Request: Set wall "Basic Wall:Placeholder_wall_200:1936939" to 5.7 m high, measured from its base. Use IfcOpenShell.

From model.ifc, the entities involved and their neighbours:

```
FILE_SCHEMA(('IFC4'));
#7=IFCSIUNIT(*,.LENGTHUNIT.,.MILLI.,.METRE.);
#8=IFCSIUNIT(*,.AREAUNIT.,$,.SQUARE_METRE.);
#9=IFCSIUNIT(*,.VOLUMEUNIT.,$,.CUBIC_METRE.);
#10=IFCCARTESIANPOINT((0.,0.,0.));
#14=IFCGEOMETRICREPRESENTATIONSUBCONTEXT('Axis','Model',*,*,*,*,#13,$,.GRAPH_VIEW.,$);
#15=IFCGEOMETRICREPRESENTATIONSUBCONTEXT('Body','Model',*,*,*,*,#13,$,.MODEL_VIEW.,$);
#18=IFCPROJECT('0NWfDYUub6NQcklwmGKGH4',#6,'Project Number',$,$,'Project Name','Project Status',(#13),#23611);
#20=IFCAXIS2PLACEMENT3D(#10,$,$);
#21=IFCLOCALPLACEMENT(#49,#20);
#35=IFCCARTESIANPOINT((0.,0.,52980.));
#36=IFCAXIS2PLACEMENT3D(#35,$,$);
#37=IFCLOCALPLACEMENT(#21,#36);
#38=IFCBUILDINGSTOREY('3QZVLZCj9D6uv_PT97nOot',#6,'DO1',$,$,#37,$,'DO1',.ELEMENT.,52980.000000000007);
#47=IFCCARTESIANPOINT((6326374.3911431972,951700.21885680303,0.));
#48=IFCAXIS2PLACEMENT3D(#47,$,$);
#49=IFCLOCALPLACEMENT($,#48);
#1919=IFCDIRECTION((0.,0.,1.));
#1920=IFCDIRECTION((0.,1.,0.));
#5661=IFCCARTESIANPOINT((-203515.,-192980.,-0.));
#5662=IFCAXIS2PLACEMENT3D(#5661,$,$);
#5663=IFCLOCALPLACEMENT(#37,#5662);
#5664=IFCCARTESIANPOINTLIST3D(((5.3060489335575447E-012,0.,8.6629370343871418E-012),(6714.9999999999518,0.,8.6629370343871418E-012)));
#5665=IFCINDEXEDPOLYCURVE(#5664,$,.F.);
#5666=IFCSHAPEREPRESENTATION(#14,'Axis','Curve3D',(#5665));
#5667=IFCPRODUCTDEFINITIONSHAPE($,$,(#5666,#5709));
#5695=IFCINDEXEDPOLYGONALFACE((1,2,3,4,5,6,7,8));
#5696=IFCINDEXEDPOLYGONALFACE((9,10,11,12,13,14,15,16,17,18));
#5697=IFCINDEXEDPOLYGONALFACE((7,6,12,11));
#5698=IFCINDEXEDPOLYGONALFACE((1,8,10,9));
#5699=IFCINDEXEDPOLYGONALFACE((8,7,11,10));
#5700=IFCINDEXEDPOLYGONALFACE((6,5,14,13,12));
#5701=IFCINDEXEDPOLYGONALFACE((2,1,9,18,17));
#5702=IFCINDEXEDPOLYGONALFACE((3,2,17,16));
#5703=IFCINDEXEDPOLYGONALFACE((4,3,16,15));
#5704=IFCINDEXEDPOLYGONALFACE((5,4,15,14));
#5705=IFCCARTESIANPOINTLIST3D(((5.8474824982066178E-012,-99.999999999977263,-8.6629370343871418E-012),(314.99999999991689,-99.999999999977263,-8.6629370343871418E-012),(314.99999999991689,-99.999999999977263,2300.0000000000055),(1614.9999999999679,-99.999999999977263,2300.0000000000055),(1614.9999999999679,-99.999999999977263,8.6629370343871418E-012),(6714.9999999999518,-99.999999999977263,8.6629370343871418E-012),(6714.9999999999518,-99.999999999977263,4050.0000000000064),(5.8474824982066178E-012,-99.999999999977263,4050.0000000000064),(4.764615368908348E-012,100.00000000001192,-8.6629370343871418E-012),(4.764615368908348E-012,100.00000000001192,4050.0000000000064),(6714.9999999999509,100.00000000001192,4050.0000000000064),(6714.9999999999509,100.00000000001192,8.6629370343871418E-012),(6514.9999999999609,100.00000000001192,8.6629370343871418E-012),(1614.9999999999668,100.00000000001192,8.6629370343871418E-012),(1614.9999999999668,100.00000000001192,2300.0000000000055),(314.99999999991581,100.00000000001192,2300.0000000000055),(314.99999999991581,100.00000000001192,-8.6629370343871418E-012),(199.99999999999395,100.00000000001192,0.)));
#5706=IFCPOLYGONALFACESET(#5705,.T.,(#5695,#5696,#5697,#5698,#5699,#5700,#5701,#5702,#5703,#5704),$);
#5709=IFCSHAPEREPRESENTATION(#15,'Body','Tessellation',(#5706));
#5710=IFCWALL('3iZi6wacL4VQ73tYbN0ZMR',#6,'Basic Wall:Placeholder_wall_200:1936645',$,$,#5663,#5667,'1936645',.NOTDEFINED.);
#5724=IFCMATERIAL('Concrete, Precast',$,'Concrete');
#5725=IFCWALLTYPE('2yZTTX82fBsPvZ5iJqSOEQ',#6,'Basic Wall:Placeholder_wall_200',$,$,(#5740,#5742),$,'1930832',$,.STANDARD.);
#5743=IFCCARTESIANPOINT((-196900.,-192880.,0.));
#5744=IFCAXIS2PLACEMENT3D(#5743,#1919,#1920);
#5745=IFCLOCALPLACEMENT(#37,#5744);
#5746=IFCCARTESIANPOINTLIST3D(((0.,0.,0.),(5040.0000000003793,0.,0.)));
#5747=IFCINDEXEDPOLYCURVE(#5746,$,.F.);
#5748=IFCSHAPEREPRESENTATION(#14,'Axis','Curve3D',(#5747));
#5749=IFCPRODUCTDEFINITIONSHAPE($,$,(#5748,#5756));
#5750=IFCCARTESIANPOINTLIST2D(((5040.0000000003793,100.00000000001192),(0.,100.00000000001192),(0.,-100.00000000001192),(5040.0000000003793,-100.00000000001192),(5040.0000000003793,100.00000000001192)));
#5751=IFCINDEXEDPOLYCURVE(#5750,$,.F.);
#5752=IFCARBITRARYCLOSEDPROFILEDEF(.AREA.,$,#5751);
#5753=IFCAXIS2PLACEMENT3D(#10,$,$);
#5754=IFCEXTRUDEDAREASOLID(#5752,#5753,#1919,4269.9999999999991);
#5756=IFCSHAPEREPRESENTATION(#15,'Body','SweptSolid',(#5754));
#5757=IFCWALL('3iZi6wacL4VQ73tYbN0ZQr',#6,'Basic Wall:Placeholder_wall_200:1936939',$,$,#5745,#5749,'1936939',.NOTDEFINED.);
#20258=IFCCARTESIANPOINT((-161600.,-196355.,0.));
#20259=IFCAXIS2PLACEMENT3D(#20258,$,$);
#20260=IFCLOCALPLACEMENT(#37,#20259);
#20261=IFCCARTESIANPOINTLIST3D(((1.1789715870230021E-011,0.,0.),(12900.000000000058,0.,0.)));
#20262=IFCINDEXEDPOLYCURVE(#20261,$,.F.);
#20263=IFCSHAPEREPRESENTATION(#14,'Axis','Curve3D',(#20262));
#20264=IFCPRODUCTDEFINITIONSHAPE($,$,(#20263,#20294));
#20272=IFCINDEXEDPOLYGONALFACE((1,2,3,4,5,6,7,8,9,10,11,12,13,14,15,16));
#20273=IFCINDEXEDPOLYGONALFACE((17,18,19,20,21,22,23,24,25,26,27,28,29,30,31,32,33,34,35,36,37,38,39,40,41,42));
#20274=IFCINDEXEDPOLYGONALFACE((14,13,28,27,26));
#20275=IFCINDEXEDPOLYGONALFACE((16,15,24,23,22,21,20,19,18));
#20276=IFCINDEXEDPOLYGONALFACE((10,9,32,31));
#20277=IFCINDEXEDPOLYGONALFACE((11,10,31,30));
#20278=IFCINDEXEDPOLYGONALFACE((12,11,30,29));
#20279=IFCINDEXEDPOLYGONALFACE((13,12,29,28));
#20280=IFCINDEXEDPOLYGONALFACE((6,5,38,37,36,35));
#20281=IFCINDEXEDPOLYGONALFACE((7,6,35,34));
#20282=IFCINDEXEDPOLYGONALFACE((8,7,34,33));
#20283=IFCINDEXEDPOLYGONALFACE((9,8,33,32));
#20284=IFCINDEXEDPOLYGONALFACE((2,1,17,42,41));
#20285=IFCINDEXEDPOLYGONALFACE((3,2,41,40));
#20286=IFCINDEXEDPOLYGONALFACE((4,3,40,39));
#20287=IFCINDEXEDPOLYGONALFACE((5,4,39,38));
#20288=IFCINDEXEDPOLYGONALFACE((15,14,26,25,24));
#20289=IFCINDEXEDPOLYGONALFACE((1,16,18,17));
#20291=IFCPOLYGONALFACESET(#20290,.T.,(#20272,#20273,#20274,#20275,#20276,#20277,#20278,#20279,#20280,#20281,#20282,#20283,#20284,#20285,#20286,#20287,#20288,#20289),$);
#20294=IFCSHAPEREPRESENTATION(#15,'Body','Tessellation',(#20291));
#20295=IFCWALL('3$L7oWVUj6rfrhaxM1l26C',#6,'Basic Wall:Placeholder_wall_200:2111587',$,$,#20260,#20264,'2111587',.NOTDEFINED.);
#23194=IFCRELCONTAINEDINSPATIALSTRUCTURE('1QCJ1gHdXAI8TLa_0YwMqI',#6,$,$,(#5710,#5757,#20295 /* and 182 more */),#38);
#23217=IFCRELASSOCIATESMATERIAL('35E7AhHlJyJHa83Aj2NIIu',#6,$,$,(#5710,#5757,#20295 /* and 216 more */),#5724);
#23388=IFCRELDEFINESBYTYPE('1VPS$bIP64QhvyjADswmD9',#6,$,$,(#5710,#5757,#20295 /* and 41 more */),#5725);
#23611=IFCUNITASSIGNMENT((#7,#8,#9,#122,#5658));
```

```python
import ifcopenshell
import ifcopenshell.geom
import ifcopenshell.util.representation
import ifcopenshell.util.shape
import ifcopenshell.util.unit

model = ifcopenshell.open("model.ifc")
unit_scale = ifcopenshell.util.unit.calculate_unit_scale(model)
settings = ifcopenshell.geom.settings()


def volume(element):
    """Net volume in cubic metres, openings subtracted."""
    shape = ifcopenshell.geom.create_shape(settings, element)
    return ifcopenshell.util.shape.get_volume(shape.geometry)


wall = model.by_guid("3iZi6wacL4VQ73tYbN0ZQr")
before = volume(wall)

body = ifcopenshell.util.representation.get_representation(wall, "Model", "Body")
solid = body.Items[0]
old_height = solid.Depth
solid.Depth = 5.7 / unit_scale
after = volume(wall)

print(f"height {old_height:g} -> {solid.Depth:g}, volume {before:.3f} -> {after:.3f} m3")

model.write("model_v2.ifc")
```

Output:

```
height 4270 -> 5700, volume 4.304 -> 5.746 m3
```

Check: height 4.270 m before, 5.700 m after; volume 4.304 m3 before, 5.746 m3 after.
